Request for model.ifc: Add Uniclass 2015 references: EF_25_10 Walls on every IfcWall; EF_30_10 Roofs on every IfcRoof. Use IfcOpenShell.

First a look at what the model holds.

```python
import ifcopenshell

model = ifcopenshell.open("model.ifc")
print(model.schema)
print("classifications:", [c.Name for c in model.by_type("IfcClassification")])
for ifc_class in ("IfcDoor", "IfcRoof", "IfcStair", "IfcWall", "IfcWindow"):
    print(ifc_class, len(model.by_type(ifc_class)))
```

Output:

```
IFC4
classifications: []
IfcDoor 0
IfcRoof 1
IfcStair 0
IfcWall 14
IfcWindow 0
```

```python
import ifcopenshell
import ifcopenshell.api.classification

model = ifcopenshell.open("model.ifc")

system = ifcopenshell.api.classification.add_classification(model, classification="Uniclass 2015")

codes = {
    "IfcWall": ("EF_25_10", "Walls"),
    "IfcRoof": ("EF_30_10", "Roofs"),
}
for ifc_class, (code, name) in codes.items():
    products = model.by_type(ifc_class)
    ifcopenshell.api.classification.add_reference(
        model, products=products, classification=system, identification=code, name=name
    )
    print(code, len(products))

model.write("model_edited.ifc")
```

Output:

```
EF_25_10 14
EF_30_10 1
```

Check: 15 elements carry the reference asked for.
